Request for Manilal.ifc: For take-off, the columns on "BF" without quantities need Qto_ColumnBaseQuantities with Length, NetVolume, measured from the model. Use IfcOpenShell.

First a look at what the model holds.

```python
import ifcopenshell
import ifcopenshell.util.element
import ifcopenshell.util.unit

model = ifcopenshell.open("Manilal.ifc")
print(model.schema)
for unit_type in ("LENGTHUNIT", "AREAUNIT", "VOLUMEUNIT"):
    print(unit_type, ifcopenshell.util.unit.calculate_unit_scale(model, unit_type))
storey = next(s for s in model.by_type("IfcBuildingStorey") if s.Name == "BF")
columns = [e for e in ifcopenshell.util.element.get_decomposition(storey) if e.is_a("IfcColumn")]
for e in sorted(columns, key=lambda e: e.id()):
    print(e.id(), e.is_a(), e.Name, list(ifcopenshell.util.element.get_psets(e, qtos_only=True)), sep=" | ")
```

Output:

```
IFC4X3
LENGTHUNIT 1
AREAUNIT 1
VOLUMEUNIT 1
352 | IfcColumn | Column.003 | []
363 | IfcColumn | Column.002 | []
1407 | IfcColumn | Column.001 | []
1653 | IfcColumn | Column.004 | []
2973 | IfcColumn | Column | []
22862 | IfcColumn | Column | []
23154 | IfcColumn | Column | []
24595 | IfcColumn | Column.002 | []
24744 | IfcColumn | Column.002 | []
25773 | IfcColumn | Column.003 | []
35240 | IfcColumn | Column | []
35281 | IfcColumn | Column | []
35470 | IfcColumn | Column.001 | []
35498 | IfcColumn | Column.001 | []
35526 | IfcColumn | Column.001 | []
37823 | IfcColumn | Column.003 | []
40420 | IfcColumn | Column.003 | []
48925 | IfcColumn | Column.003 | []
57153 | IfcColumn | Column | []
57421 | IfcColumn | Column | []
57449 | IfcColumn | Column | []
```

```python
import ifcopenshell
import ifcopenshell.api.pset
import ifcopenshell.geom
import ifcopenshell.util.element
import ifcopenshell.util.shape
import ifcopenshell.util.unit

model = ifcopenshell.open("Manilal.ifc")
unit_scale = ifcopenshell.util.unit.calculate_unit_scale(model)
volume_scale = ifcopenshell.util.unit.calculate_unit_scale(model, "VOLUMEUNIT")
settings = ifcopenshell.geom.settings()

storey = next(s for s in model.by_type("IfcBuildingStorey") if s.Name == "BF")
columns = [e for e in ifcopenshell.util.element.get_decomposition(storey) if e.is_a("IfcColumn")]

for e in sorted(columns, key=lambda e: e.id()):
    if ifcopenshell.util.element.get_psets(e, qtos_only=True, should_inherit=False):
        continue
    # Geometry comes back in metres, in the element's own axes.
    shape = ifcopenshell.geom.create_shape(settings, e)
    values = {
        "Length": ifcopenshell.util.shape.get_z(shape.geometry) / unit_scale,
        "NetVolume": ifcopenshell.util.shape.get_volume(shape.geometry) / volume_scale,
    }
    qto = ifcopenshell.api.pset.add_qto(model, product=e, name="Qto_ColumnBaseQuantities")
    ifcopenshell.api.pset.edit_qto(model, qto=qto, properties=values)
    print(e.id(), {k: round(v, 3) for k, v in values.items()})

model.write("Manilal_updated.ifc")
```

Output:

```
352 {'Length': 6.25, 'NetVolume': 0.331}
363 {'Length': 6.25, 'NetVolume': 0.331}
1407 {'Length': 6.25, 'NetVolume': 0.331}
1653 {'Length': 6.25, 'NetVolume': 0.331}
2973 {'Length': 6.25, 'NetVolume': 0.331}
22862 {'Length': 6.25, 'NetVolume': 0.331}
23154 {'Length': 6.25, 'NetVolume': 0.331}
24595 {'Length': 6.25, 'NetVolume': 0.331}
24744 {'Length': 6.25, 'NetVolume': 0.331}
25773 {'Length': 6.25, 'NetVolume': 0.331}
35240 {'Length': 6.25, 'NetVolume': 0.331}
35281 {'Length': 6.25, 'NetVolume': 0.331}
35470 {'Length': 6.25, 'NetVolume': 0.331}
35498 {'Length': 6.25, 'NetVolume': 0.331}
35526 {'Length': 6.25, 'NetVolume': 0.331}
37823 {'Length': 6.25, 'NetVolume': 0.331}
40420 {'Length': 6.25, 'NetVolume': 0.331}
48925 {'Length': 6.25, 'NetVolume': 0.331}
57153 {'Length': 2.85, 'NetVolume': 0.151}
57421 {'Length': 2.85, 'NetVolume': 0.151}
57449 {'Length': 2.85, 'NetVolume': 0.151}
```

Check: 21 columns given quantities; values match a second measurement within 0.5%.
